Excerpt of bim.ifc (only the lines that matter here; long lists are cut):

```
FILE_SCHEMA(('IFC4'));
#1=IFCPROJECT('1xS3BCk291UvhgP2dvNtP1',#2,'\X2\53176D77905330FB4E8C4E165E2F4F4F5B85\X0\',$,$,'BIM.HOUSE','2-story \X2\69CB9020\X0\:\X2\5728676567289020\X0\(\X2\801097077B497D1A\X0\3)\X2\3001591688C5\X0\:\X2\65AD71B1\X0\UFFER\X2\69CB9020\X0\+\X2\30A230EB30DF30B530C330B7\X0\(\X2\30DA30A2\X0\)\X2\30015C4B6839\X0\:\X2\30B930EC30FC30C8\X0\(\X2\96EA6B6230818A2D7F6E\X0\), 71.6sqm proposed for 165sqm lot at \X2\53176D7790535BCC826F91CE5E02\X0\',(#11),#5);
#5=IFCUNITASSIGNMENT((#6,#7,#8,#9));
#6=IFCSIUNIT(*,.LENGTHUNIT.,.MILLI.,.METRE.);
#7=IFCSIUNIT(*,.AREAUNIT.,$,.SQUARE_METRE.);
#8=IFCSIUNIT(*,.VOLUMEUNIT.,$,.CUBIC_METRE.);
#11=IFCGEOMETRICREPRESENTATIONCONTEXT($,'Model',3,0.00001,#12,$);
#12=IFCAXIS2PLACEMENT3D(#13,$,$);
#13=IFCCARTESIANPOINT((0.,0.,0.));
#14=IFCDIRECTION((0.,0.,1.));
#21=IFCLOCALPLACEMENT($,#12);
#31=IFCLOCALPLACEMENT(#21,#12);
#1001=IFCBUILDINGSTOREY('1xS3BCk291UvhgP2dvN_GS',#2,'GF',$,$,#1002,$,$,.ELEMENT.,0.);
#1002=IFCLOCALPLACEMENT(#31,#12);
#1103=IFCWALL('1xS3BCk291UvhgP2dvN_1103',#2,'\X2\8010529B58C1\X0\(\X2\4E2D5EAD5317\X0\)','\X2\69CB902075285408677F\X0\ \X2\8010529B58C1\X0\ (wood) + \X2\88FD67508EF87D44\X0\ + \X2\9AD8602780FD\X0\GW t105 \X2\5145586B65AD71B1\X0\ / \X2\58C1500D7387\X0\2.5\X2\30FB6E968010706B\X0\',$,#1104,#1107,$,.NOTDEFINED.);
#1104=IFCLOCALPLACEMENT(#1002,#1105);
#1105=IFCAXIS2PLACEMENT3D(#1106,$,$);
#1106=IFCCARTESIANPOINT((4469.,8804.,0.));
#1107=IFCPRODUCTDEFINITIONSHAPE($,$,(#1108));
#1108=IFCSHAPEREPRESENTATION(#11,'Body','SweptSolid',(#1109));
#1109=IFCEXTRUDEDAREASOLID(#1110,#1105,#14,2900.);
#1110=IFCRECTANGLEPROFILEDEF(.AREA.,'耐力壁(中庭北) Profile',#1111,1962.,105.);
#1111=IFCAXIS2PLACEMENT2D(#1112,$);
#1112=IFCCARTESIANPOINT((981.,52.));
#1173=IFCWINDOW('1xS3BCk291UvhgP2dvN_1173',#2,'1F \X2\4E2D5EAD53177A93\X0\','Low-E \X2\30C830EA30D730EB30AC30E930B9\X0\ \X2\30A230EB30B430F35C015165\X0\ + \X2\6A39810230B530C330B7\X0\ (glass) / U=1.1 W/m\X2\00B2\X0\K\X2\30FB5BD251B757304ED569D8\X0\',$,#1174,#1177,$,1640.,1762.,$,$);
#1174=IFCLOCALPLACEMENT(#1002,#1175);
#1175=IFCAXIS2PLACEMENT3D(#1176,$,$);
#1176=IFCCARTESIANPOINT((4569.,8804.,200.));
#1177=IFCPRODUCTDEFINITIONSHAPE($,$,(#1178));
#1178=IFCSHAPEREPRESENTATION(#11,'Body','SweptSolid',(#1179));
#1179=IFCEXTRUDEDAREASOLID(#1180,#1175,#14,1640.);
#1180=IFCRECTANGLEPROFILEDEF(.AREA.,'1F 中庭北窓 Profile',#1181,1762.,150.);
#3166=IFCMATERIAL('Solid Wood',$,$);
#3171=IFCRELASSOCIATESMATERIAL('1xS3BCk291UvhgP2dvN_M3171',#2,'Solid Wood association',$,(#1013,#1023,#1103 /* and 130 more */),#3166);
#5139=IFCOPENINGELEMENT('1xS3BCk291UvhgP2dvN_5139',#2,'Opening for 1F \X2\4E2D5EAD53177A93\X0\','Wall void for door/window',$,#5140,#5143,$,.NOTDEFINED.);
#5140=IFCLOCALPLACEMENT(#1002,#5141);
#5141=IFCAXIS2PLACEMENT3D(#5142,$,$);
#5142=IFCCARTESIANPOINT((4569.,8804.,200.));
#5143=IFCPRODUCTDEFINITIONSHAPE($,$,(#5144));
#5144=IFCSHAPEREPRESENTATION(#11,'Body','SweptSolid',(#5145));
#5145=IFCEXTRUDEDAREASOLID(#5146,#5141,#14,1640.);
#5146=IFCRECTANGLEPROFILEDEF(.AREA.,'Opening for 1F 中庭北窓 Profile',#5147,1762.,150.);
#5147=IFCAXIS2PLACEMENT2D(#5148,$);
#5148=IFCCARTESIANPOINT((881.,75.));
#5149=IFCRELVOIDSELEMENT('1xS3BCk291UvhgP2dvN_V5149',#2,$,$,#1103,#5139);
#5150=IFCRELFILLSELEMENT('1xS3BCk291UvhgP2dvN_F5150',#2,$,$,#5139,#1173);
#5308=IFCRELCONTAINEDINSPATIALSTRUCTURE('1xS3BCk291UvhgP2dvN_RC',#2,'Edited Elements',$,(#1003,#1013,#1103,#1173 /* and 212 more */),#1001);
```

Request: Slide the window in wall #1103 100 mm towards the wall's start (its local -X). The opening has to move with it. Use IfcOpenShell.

```python
import ifcopenshell
import ifcopenshell.api.geometry
import ifcopenshell.util.placement
import ifcopenshell.util.unit

model = ifcopenshell.open("bim.ifc")
unit_scale = ifcopenshell.util.unit.calculate_unit_scale(model)

window = model.by_guid("1xS3BCk291UvhgP2dvN_1173")
opening = window.FillsVoids[0].RelatingOpeningElement
wall = opening.VoidsElements[0].RelatingBuildingElement

wall_matrix = ifcopenshell.util.placement.get_local_placement(wall.ObjectPlacement)
shift = wall_matrix[:3, 0] * -0.1 / unit_scale
before = ifcopenshell.util.placement.get_local_placement(window.ObjectPlacement)[:3, 3].copy()

# The window is not placed relative to its opening, so move both.
for product in (opening, window):
    matrix = ifcopenshell.util.placement.get_local_placement(product.ObjectPlacement)
    matrix[:3, 3] += shift
    ifcopenshell.api.geometry.edit_object_placement(model, product=product, matrix=matrix, is_si=False)

after = ifcopenshell.util.placement.get_local_placement(window.ObjectPlacement)[:3, 3]
print("window moved by", (after - before).round(3) + 0.0)

model.write("bim_rev.ifc")
```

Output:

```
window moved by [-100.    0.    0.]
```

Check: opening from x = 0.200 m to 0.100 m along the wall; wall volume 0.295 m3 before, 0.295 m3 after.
